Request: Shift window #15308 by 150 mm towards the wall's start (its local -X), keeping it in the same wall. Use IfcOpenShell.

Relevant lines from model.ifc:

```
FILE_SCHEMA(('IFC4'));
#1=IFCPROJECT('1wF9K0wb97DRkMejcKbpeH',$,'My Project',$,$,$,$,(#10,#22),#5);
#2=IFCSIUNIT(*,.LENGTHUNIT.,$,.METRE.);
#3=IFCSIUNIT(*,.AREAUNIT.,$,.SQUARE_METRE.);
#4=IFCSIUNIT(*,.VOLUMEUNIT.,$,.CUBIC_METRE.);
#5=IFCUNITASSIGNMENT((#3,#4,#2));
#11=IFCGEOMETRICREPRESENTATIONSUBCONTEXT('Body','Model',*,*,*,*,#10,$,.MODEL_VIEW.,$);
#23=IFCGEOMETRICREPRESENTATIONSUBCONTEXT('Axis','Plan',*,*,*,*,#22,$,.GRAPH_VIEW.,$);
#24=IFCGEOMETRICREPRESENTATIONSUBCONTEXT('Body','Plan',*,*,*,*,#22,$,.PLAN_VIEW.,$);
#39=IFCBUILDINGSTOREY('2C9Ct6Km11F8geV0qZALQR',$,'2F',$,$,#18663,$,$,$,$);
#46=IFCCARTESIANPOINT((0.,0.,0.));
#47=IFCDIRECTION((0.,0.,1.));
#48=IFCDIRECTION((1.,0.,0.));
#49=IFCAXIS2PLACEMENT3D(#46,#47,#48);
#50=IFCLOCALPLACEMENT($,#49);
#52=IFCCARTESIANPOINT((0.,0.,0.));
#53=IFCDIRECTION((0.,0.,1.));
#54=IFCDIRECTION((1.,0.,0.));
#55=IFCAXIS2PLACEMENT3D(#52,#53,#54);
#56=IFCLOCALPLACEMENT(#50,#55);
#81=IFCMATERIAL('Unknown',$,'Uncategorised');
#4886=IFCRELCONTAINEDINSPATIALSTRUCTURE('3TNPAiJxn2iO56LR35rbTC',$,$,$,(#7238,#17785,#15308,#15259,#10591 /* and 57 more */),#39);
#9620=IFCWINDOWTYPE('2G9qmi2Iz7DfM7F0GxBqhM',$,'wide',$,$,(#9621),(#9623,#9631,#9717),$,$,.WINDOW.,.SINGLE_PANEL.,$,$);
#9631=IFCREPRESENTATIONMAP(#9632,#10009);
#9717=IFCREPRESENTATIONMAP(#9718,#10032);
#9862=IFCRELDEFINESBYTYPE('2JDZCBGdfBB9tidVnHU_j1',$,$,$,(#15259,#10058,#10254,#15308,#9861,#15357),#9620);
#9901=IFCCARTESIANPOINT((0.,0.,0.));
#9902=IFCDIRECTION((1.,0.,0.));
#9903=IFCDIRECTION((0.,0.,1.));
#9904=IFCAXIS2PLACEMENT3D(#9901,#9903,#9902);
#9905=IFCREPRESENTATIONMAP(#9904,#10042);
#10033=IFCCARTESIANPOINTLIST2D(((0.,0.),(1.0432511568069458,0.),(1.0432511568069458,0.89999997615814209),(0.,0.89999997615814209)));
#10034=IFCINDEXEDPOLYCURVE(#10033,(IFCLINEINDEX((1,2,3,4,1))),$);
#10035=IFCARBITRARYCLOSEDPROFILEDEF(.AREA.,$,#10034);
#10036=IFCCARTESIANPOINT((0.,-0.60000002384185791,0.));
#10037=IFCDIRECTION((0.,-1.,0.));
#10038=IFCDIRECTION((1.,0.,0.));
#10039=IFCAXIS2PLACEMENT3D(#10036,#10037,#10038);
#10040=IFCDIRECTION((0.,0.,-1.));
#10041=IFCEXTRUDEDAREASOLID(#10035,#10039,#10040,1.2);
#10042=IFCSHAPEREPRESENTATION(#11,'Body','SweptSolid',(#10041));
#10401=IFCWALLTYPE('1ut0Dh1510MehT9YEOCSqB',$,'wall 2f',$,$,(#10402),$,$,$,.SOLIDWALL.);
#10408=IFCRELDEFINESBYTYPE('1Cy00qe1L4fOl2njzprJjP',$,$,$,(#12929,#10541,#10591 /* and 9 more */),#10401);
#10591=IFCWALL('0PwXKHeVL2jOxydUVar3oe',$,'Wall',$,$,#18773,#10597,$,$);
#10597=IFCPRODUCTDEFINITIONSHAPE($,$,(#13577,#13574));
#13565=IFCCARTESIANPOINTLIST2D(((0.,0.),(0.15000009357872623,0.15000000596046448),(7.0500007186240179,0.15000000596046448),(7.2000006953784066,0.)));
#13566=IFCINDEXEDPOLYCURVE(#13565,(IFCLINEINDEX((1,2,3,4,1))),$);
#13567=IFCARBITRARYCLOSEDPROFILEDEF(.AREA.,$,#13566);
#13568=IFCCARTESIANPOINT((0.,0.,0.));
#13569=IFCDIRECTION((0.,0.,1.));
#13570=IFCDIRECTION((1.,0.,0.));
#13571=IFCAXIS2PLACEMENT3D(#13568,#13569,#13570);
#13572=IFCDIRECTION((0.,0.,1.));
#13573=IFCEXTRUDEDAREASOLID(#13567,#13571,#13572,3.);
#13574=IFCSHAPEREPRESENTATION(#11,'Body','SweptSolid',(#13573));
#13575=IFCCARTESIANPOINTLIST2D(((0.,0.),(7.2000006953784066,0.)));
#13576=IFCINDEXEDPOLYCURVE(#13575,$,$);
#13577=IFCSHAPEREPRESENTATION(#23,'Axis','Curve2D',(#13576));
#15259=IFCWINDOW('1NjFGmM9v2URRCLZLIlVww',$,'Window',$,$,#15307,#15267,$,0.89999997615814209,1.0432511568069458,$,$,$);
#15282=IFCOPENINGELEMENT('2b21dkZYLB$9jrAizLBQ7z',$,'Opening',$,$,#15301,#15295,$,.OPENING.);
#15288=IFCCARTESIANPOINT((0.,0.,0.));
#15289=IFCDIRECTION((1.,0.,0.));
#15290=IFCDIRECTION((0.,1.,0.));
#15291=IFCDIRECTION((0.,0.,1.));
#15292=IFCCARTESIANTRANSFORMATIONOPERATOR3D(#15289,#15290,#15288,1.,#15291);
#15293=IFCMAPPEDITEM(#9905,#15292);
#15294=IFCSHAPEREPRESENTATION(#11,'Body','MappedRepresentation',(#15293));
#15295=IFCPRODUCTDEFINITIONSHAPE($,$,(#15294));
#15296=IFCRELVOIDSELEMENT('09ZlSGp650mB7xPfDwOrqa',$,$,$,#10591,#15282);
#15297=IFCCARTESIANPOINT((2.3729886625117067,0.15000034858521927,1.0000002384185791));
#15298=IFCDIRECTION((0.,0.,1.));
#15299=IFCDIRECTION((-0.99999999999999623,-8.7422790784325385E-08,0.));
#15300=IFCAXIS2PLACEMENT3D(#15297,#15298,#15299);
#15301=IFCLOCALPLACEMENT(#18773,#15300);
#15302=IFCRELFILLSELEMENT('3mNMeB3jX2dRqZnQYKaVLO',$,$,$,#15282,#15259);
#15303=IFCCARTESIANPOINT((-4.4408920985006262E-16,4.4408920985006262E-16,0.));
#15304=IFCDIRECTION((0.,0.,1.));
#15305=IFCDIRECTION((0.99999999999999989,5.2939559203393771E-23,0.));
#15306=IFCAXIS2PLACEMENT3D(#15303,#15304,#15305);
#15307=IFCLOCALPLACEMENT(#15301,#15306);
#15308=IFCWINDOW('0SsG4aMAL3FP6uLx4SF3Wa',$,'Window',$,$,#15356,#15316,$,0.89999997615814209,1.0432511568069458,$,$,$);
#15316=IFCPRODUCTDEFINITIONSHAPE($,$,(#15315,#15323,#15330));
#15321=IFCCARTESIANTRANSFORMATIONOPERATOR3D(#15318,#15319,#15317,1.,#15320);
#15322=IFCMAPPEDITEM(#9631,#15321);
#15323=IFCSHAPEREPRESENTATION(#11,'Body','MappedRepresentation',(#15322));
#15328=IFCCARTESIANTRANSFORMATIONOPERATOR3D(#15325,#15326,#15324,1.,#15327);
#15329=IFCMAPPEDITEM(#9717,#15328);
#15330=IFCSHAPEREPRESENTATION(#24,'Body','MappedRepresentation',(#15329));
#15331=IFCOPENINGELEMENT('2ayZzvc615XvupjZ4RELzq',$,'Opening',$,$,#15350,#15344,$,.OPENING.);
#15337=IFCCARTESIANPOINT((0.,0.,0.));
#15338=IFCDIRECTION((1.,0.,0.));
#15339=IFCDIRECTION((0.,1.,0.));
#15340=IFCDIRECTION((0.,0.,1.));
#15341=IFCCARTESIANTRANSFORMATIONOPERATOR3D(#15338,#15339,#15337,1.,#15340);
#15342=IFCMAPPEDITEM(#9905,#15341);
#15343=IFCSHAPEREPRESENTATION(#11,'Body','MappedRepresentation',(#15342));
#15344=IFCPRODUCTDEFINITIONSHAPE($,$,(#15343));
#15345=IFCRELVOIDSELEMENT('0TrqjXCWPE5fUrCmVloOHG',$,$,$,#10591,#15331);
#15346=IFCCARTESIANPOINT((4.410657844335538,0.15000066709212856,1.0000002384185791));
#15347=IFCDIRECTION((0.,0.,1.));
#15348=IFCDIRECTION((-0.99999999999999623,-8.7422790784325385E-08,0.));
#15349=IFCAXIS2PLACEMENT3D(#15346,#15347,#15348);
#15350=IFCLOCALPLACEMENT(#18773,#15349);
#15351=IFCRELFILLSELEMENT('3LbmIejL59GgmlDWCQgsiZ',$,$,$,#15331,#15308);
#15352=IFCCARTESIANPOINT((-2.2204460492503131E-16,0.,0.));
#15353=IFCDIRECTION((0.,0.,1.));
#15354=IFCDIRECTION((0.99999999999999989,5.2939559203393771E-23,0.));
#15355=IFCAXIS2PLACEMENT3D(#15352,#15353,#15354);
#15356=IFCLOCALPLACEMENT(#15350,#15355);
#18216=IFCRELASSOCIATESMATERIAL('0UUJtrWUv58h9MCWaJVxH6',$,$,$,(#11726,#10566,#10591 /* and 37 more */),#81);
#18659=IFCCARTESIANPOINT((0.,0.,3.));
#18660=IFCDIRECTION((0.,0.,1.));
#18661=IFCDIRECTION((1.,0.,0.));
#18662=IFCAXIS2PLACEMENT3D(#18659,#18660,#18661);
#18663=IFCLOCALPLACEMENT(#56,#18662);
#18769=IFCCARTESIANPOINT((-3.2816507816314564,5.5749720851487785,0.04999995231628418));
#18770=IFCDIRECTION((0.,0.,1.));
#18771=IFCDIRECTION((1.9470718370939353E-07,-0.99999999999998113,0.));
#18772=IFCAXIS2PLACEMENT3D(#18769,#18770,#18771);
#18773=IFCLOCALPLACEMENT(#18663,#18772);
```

```python
import ifcopenshell
import ifcopenshell.api.geometry
import ifcopenshell.util.placement
import ifcopenshell.util.unit

model = ifcopenshell.open("model.ifc")
unit_scale = ifcopenshell.util.unit.calculate_unit_scale(model)

window = model.by_guid("0SsG4aMAL3FP6uLx4SF3Wa")
opening = window.FillsVoids[0].RelatingOpeningElement
wall = opening.VoidsElements[0].RelatingBuildingElement

wall_matrix = ifcopenshell.util.placement.get_local_placement(wall.ObjectPlacement)
shift = wall_matrix[:3, 0] * -0.15 / unit_scale
before = ifcopenshell.util.placement.get_local_placement(window.ObjectPlacement)[:3, 3].copy()

# The window is placed relative to its opening, so it follows when the opening moves.
matrix = ifcopenshell.util.placement.get_local_placement(opening.ObjectPlacement)
matrix[:3, 3] += shift
ifcopenshell.api.geometry.edit_object_placement(
    model, product=opening, matrix=matrix, is_si=False, should_transform_children=True
)

after = ifcopenshell.util.placement.get_local_placement(window.ObjectPlacement)[:3, 3]
print("window moved by", (after - before).round(3) + 0.0)

model.write("model_edited.ifc")
```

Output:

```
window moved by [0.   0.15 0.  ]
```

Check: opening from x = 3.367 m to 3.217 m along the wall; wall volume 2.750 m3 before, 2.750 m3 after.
